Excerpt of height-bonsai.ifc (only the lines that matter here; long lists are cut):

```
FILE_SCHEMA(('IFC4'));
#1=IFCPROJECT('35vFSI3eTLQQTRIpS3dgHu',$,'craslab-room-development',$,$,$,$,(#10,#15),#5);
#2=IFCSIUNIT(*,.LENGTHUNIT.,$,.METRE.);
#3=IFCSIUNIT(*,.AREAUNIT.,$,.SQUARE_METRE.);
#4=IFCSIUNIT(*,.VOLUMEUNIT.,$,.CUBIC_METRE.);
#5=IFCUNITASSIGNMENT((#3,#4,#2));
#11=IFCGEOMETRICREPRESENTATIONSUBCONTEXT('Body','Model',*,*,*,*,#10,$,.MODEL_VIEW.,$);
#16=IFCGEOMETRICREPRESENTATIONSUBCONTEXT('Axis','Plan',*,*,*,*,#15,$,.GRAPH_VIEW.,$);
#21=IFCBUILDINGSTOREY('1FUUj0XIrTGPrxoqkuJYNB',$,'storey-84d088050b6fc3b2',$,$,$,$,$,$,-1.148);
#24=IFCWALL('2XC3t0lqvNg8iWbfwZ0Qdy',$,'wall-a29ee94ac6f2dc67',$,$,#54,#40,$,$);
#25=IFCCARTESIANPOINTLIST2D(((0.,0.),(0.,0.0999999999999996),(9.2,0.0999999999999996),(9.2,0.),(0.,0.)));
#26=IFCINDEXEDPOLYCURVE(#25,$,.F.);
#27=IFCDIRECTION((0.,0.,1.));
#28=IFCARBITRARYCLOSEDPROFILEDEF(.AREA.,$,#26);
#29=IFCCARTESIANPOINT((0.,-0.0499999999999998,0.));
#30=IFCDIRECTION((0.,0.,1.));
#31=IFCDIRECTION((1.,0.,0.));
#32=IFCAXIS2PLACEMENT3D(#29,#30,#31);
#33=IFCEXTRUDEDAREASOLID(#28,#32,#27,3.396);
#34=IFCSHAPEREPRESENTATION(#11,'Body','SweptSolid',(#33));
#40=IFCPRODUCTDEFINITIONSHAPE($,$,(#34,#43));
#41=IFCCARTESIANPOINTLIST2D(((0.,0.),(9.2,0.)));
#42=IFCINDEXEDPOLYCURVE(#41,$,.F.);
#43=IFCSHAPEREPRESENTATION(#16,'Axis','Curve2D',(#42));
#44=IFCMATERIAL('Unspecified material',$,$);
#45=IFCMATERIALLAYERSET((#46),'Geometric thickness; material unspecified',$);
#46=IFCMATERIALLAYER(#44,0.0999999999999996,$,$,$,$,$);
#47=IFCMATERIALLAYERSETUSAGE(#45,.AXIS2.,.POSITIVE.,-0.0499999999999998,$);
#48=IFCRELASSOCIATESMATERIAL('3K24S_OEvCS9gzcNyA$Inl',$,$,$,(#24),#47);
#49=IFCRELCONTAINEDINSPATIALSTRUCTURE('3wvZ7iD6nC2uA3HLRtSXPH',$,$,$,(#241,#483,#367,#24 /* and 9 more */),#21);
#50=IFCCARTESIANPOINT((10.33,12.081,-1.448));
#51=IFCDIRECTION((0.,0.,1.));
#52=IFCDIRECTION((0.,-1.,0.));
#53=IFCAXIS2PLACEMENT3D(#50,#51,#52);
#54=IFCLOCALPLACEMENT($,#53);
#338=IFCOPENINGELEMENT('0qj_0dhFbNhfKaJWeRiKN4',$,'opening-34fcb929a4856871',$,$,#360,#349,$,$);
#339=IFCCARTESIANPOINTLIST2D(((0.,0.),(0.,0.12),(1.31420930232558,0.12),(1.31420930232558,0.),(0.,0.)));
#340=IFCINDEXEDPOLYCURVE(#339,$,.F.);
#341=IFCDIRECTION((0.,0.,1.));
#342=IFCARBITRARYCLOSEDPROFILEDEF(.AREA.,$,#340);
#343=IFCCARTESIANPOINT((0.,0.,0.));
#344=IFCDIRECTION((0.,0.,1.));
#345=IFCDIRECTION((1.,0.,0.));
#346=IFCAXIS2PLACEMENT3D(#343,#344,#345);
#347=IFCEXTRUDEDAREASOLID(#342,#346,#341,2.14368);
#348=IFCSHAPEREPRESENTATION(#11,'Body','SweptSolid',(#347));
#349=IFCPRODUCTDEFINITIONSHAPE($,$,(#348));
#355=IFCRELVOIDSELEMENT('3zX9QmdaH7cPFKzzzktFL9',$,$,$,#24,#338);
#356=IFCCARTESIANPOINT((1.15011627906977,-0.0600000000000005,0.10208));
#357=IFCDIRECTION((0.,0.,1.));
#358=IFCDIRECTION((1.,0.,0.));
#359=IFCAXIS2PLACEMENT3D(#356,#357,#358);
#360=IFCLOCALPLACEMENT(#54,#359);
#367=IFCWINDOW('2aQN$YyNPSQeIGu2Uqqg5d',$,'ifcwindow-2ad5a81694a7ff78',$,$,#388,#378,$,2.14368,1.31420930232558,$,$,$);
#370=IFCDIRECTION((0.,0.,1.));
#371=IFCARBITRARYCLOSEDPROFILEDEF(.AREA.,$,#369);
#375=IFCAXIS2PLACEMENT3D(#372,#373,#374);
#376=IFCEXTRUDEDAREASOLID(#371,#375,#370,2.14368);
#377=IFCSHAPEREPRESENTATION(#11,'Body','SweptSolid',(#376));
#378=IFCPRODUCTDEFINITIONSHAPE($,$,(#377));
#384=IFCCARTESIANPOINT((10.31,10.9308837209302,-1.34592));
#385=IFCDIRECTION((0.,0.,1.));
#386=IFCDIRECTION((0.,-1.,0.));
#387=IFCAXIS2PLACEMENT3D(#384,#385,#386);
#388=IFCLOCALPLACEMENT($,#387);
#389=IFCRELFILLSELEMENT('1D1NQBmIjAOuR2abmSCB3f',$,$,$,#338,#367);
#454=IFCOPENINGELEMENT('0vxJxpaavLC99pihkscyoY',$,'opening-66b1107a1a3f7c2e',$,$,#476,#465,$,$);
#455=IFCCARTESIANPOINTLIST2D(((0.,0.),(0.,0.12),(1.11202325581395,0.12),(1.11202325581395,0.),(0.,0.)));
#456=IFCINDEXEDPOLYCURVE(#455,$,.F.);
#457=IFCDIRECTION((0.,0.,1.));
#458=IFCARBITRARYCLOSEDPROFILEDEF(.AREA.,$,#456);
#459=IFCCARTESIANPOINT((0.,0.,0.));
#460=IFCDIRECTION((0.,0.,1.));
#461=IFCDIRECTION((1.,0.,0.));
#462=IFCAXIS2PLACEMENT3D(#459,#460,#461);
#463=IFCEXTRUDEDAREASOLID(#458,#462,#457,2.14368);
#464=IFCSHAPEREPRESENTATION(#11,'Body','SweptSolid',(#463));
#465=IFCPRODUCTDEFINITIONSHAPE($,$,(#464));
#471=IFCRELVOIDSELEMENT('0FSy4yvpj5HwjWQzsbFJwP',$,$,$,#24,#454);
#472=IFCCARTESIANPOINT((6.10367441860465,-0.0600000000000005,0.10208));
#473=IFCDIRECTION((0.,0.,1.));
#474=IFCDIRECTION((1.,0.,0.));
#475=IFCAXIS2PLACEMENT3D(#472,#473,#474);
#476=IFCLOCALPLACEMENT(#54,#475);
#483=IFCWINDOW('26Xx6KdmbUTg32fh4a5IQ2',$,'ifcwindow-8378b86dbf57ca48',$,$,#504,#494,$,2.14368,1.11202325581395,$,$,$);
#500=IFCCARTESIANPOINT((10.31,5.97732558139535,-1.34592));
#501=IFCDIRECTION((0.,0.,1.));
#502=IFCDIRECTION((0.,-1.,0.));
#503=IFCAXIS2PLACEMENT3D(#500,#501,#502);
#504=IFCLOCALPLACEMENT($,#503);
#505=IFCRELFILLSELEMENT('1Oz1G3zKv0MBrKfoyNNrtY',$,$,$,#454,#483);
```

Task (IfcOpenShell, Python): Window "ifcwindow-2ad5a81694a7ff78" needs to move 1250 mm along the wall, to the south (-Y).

```python
import ifcopenshell
import ifcopenshell.api.geometry
import ifcopenshell.util.placement

model = ifcopenshell.open("height-bonsai.ifc")

window = model.by_guid("2aQN$YyNPSQeIGu2Uqqg5d")
opening = window.FillsVoids[0].RelatingOpeningElement
wall = opening.VoidsElements[0].RelatingBuildingElement

wall_matrix = ifcopenshell.util.placement.get_local_placement(wall.ObjectPlacement)
shift = wall_matrix[:3, 0] * 1.25
before = ifcopenshell.util.placement.get_local_placement(window.ObjectPlacement)[:3, 3].copy()

# The window is not placed relative to its opening, so move both.
for product in (opening, window):
    matrix = ifcopenshell.util.placement.get_local_placement(product.ObjectPlacement)
    matrix[:3, 3] += shift
    ifcopenshell.api.geometry.edit_object_placement(model, product=product, matrix=matrix, is_si=False)

after = ifcopenshell.util.placement.get_local_placement(window.ObjectPlacement)[:3, 3]
print("window moved by", (after - before).round(3) + 0.0)

model.write("height-bonsai-out.ifc")
```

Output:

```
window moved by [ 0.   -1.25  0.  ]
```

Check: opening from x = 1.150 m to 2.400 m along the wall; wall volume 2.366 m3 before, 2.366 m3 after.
